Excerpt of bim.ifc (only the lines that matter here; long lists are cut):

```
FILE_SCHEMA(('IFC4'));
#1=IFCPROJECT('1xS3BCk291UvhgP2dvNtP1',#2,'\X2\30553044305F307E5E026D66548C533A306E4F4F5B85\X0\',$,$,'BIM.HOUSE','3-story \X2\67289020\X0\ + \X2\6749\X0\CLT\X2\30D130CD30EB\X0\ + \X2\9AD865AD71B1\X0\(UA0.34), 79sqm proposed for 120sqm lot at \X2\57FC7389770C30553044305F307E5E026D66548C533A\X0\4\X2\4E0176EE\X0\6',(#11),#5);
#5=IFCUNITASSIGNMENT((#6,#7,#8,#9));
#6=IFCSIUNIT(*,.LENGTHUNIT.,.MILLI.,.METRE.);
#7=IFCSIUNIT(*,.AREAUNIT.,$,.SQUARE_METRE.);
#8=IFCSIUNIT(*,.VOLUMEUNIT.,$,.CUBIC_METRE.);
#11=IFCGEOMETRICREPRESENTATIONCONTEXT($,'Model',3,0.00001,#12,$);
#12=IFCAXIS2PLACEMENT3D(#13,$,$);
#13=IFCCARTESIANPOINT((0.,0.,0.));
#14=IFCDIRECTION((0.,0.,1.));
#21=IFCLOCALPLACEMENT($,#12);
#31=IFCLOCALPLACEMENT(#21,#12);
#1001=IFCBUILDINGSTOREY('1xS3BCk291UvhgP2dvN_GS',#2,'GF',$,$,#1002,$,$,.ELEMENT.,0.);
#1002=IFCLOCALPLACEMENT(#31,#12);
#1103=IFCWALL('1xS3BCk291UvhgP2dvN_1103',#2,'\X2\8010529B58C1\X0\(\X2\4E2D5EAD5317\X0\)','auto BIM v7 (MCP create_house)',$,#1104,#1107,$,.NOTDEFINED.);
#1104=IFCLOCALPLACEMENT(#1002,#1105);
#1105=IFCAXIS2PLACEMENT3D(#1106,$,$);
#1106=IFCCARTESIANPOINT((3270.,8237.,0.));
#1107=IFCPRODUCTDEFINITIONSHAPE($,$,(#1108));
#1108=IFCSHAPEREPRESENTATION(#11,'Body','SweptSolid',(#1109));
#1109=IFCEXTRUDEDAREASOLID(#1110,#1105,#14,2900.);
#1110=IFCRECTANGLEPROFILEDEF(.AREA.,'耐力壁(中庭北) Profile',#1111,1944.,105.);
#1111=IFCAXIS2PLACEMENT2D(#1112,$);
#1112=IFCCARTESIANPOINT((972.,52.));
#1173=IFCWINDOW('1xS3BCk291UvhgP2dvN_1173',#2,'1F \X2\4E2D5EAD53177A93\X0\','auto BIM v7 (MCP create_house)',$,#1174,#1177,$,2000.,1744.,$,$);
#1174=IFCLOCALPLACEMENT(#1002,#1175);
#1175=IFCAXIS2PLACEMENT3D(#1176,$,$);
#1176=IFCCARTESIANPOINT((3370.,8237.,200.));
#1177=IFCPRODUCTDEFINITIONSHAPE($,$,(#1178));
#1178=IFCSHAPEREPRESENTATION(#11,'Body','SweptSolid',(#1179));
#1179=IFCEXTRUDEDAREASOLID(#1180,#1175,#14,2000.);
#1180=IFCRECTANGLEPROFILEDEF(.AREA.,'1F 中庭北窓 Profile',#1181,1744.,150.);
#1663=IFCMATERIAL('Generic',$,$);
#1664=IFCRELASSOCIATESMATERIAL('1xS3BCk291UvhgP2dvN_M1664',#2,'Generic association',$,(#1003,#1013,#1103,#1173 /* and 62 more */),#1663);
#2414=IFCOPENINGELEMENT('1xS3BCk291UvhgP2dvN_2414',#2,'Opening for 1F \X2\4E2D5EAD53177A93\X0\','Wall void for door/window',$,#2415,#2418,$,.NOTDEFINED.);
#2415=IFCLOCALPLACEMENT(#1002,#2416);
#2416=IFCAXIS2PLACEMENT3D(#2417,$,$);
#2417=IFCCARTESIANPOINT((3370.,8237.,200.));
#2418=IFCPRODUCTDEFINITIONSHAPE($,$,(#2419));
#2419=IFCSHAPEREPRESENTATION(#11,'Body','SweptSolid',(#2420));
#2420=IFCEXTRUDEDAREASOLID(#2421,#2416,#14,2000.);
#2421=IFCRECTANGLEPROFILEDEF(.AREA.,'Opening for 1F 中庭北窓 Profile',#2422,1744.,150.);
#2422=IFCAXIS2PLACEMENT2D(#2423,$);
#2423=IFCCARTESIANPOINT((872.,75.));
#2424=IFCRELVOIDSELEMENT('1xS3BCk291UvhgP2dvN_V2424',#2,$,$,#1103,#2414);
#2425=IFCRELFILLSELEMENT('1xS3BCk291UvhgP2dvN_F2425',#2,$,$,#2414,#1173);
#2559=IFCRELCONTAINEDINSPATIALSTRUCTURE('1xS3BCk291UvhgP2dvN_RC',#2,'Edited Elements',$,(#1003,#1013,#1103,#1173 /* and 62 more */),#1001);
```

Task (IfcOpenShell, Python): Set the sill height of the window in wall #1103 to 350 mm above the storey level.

```python
import numpy as np
import ifcopenshell
import ifcopenshell.api.geometry
import ifcopenshell.geom
import ifcopenshell.util.element
import ifcopenshell.util.placement
import ifcopenshell.util.shape
import ifcopenshell.util.unit

model = ifcopenshell.open("bim.ifc")
unit_scale = ifcopenshell.util.unit.calculate_unit_scale(model)

window = model.by_guid("1xS3BCk291UvhgP2dvN_1173")
opening = window.FillsVoids[0].RelatingOpeningElement
storey = ifcopenshell.util.element.get_container(window, ifc_class="IfcBuildingStorey")
level = ifcopenshell.util.placement.get_local_placement(storey.ObjectPlacement)[2, 3]

# The opening's origin need not be at the sill, so measure its lowest point.
shape = ifcopenshell.geom.create_shape(ifcopenshell.geom.settings(), opening)
bottom = ifcopenshell.util.shape.get_shape_bottom_elevation(shape, shape.geometry) / unit_scale
dz = level + 350.0 - bottom

shift = np.array([0.0, 0.0, dz])
# The window is not placed relative to its opening, so move both.
for product in (opening, window):
    matrix = ifcopenshell.util.placement.get_local_placement(product.ObjectPlacement)
    matrix[:3, 3] += shift
    ifcopenshell.api.geometry.edit_object_placement(model, product=product, matrix=matrix, is_si=False)

print(f"moved by {dz * unit_scale:+.3f} m")

model.write("bim_edited.ifc")
```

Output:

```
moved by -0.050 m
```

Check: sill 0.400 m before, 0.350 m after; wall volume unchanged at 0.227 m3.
